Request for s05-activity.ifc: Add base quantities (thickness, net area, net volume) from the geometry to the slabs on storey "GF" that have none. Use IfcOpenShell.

First a look at what the model holds.

```python
import ifcopenshell
import ifcopenshell.util.element
import ifcopenshell.util.unit

model = ifcopenshell.open("s05-activity.ifc")
print(model.schema)
for unit_type in ("LENGTHUNIT", "AREAUNIT", "VOLUMEUNIT"):
    print(unit_type, ifcopenshell.util.unit.calculate_unit_scale(model, unit_type))
storey = next(s for s in model.by_type("IfcBuildingStorey") if s.Name == "GF")
slabs = [e for e in ifcopenshell.util.element.get_decomposition(storey) if e.is_a("IfcSlab")]
for e in sorted(slabs, key=lambda e: e.id()):
    print(e.id(), e.is_a(), e.Name, list(ifcopenshell.util.element.get_psets(e, qtos_only=True)), sep=" | ")
```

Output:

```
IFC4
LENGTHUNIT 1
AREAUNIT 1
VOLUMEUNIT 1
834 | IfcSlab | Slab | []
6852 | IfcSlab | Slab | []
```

```python
import ifcopenshell
import ifcopenshell.api.pset
import ifcopenshell.geom
import ifcopenshell.util.element
import ifcopenshell.util.shape
import ifcopenshell.util.unit

model = ifcopenshell.open("s05-activity.ifc")
unit_scale = ifcopenshell.util.unit.calculate_unit_scale(model)
area_scale = ifcopenshell.util.unit.calculate_unit_scale(model, "AREAUNIT")
volume_scale = ifcopenshell.util.unit.calculate_unit_scale(model, "VOLUMEUNIT")
settings = ifcopenshell.geom.settings()

storey = next(s for s in model.by_type("IfcBuildingStorey") if s.Name == "GF")
slabs = [e for e in ifcopenshell.util.element.get_decomposition(storey) if e.is_a("IfcSlab")]

for e in sorted(slabs, key=lambda e: e.id()):
    if ifcopenshell.util.element.get_psets(e, qtos_only=True, should_inherit=False):
        continue
    # Geometry comes back in metres, in the element's own axes.
    shape = ifcopenshell.geom.create_shape(settings, e)
    values = {
        "Width": ifcopenshell.util.shape.get_z(shape.geometry) / unit_scale,
        "NetArea": ifcopenshell.util.shape.get_footprint_area(shape.geometry) / area_scale,
        "NetVolume": ifcopenshell.util.shape.get_volume(shape.geometry) / volume_scale,
    }
    qto = ifcopenshell.api.pset.add_qto(model, product=e, name="Qto_SlabBaseQuantities")
    ifcopenshell.api.pset.edit_qto(model, qto=qto, properties=values)
    print(e.id(), {k: round(v, 3) for k, v in values.items()})

model.write("s05-activity_edited.ifc")
```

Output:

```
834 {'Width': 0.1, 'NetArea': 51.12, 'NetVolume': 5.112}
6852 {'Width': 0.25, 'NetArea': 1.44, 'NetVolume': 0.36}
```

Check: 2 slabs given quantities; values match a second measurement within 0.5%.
